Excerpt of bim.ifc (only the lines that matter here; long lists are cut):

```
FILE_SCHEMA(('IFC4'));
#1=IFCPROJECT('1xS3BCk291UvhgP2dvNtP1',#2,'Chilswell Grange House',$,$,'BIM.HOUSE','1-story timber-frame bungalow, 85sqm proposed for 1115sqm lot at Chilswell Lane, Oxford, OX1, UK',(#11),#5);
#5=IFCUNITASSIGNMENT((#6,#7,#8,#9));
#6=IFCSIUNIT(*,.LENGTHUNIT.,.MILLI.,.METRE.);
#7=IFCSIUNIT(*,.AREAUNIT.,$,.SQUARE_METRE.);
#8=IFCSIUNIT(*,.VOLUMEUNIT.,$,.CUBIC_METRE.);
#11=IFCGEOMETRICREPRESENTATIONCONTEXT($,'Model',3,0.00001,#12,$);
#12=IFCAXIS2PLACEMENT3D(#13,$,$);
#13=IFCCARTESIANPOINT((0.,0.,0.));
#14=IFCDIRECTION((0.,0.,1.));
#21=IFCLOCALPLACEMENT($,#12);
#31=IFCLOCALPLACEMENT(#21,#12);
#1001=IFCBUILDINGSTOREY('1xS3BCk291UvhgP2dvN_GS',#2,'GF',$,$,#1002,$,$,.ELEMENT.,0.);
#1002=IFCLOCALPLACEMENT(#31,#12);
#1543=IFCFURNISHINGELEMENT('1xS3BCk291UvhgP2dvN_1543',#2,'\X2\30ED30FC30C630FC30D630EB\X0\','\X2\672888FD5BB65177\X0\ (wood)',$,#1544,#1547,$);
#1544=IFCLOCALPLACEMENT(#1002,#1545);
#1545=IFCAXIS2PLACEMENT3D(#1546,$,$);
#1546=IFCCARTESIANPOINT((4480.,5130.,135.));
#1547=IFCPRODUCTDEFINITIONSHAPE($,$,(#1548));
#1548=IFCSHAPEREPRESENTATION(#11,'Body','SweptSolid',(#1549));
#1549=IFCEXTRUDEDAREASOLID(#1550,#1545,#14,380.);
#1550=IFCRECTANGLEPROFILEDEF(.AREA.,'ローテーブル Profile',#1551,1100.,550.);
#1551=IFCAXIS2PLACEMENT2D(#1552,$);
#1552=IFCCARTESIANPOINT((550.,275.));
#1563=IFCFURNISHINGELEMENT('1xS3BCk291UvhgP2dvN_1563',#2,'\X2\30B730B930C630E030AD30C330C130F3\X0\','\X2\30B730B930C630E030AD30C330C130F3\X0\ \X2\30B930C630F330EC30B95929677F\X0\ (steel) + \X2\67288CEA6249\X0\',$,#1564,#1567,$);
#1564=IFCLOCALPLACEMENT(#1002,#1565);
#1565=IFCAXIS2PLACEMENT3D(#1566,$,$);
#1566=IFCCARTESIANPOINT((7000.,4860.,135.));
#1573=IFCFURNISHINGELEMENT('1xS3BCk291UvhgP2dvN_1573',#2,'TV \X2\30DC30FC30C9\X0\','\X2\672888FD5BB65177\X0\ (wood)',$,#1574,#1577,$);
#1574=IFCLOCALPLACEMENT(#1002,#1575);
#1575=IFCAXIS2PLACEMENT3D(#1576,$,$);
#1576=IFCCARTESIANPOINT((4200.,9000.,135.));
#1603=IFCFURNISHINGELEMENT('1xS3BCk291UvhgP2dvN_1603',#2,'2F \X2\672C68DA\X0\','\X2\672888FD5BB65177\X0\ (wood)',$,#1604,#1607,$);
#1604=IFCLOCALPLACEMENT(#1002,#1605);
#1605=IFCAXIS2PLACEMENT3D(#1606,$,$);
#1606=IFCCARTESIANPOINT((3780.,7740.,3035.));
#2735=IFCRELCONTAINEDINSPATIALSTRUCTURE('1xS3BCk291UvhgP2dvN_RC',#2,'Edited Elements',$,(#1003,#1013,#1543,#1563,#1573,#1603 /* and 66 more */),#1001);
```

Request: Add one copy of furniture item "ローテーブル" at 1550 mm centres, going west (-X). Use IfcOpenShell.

```python
import numpy as np
import ifcopenshell
import ifcopenshell.api.geometry
import ifcopenshell.api.root
import ifcopenshell.util.element
import ifcopenshell.util.placement
import ifcopenshell.util.unit

model = ifcopenshell.open("bim.ifc")
unit_scale = ifcopenshell.util.unit.calculate_unit_scale(model)


def reuse_history(source, copy):
    """copy_class also copies each property set's owner history, people and application; keep the originals."""
    for rel in copy.IsDefinedBy:
        if rel.is_a("IfcRelDefinesByProperties") and (history := rel.RelatingPropertyDefinition.OwnerHistory):
            rel.RelatingPropertyDefinition.OwnerHistory = source.OwnerHistory
            ifcopenshell.util.element.remove_deep2(model, history)


source = model.by_guid("1xS3BCk291UvhgP2dvN_1543")
base = ifcopenshell.util.placement.get_local_placement(source.ObjectPlacement)
step = np.array([-1.0, 0.0, 0.0]) * 1.55 / unit_scale

for i in range(1, 2):
    copy = ifcopenshell.api.root.copy_class(model, product=source)
    copy.Representation = ifcopenshell.util.element.copy_deep(
        model, source.Representation, exclude=["IfcGeometricRepresentationContext", "IfcRepresentationMap"]
    )
    reuse_history(source, copy)
    matrix = base.copy()
    matrix[:3, 3] += i * step
    print("added at", matrix[:3, 3].round(3) + 0.0)
    ifcopenshell.api.geometry.edit_object_placement(model, product=copy, matrix=matrix, is_si=False)

model.write("bim_updated.ifc")
```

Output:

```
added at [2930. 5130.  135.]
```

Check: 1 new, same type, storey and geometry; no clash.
